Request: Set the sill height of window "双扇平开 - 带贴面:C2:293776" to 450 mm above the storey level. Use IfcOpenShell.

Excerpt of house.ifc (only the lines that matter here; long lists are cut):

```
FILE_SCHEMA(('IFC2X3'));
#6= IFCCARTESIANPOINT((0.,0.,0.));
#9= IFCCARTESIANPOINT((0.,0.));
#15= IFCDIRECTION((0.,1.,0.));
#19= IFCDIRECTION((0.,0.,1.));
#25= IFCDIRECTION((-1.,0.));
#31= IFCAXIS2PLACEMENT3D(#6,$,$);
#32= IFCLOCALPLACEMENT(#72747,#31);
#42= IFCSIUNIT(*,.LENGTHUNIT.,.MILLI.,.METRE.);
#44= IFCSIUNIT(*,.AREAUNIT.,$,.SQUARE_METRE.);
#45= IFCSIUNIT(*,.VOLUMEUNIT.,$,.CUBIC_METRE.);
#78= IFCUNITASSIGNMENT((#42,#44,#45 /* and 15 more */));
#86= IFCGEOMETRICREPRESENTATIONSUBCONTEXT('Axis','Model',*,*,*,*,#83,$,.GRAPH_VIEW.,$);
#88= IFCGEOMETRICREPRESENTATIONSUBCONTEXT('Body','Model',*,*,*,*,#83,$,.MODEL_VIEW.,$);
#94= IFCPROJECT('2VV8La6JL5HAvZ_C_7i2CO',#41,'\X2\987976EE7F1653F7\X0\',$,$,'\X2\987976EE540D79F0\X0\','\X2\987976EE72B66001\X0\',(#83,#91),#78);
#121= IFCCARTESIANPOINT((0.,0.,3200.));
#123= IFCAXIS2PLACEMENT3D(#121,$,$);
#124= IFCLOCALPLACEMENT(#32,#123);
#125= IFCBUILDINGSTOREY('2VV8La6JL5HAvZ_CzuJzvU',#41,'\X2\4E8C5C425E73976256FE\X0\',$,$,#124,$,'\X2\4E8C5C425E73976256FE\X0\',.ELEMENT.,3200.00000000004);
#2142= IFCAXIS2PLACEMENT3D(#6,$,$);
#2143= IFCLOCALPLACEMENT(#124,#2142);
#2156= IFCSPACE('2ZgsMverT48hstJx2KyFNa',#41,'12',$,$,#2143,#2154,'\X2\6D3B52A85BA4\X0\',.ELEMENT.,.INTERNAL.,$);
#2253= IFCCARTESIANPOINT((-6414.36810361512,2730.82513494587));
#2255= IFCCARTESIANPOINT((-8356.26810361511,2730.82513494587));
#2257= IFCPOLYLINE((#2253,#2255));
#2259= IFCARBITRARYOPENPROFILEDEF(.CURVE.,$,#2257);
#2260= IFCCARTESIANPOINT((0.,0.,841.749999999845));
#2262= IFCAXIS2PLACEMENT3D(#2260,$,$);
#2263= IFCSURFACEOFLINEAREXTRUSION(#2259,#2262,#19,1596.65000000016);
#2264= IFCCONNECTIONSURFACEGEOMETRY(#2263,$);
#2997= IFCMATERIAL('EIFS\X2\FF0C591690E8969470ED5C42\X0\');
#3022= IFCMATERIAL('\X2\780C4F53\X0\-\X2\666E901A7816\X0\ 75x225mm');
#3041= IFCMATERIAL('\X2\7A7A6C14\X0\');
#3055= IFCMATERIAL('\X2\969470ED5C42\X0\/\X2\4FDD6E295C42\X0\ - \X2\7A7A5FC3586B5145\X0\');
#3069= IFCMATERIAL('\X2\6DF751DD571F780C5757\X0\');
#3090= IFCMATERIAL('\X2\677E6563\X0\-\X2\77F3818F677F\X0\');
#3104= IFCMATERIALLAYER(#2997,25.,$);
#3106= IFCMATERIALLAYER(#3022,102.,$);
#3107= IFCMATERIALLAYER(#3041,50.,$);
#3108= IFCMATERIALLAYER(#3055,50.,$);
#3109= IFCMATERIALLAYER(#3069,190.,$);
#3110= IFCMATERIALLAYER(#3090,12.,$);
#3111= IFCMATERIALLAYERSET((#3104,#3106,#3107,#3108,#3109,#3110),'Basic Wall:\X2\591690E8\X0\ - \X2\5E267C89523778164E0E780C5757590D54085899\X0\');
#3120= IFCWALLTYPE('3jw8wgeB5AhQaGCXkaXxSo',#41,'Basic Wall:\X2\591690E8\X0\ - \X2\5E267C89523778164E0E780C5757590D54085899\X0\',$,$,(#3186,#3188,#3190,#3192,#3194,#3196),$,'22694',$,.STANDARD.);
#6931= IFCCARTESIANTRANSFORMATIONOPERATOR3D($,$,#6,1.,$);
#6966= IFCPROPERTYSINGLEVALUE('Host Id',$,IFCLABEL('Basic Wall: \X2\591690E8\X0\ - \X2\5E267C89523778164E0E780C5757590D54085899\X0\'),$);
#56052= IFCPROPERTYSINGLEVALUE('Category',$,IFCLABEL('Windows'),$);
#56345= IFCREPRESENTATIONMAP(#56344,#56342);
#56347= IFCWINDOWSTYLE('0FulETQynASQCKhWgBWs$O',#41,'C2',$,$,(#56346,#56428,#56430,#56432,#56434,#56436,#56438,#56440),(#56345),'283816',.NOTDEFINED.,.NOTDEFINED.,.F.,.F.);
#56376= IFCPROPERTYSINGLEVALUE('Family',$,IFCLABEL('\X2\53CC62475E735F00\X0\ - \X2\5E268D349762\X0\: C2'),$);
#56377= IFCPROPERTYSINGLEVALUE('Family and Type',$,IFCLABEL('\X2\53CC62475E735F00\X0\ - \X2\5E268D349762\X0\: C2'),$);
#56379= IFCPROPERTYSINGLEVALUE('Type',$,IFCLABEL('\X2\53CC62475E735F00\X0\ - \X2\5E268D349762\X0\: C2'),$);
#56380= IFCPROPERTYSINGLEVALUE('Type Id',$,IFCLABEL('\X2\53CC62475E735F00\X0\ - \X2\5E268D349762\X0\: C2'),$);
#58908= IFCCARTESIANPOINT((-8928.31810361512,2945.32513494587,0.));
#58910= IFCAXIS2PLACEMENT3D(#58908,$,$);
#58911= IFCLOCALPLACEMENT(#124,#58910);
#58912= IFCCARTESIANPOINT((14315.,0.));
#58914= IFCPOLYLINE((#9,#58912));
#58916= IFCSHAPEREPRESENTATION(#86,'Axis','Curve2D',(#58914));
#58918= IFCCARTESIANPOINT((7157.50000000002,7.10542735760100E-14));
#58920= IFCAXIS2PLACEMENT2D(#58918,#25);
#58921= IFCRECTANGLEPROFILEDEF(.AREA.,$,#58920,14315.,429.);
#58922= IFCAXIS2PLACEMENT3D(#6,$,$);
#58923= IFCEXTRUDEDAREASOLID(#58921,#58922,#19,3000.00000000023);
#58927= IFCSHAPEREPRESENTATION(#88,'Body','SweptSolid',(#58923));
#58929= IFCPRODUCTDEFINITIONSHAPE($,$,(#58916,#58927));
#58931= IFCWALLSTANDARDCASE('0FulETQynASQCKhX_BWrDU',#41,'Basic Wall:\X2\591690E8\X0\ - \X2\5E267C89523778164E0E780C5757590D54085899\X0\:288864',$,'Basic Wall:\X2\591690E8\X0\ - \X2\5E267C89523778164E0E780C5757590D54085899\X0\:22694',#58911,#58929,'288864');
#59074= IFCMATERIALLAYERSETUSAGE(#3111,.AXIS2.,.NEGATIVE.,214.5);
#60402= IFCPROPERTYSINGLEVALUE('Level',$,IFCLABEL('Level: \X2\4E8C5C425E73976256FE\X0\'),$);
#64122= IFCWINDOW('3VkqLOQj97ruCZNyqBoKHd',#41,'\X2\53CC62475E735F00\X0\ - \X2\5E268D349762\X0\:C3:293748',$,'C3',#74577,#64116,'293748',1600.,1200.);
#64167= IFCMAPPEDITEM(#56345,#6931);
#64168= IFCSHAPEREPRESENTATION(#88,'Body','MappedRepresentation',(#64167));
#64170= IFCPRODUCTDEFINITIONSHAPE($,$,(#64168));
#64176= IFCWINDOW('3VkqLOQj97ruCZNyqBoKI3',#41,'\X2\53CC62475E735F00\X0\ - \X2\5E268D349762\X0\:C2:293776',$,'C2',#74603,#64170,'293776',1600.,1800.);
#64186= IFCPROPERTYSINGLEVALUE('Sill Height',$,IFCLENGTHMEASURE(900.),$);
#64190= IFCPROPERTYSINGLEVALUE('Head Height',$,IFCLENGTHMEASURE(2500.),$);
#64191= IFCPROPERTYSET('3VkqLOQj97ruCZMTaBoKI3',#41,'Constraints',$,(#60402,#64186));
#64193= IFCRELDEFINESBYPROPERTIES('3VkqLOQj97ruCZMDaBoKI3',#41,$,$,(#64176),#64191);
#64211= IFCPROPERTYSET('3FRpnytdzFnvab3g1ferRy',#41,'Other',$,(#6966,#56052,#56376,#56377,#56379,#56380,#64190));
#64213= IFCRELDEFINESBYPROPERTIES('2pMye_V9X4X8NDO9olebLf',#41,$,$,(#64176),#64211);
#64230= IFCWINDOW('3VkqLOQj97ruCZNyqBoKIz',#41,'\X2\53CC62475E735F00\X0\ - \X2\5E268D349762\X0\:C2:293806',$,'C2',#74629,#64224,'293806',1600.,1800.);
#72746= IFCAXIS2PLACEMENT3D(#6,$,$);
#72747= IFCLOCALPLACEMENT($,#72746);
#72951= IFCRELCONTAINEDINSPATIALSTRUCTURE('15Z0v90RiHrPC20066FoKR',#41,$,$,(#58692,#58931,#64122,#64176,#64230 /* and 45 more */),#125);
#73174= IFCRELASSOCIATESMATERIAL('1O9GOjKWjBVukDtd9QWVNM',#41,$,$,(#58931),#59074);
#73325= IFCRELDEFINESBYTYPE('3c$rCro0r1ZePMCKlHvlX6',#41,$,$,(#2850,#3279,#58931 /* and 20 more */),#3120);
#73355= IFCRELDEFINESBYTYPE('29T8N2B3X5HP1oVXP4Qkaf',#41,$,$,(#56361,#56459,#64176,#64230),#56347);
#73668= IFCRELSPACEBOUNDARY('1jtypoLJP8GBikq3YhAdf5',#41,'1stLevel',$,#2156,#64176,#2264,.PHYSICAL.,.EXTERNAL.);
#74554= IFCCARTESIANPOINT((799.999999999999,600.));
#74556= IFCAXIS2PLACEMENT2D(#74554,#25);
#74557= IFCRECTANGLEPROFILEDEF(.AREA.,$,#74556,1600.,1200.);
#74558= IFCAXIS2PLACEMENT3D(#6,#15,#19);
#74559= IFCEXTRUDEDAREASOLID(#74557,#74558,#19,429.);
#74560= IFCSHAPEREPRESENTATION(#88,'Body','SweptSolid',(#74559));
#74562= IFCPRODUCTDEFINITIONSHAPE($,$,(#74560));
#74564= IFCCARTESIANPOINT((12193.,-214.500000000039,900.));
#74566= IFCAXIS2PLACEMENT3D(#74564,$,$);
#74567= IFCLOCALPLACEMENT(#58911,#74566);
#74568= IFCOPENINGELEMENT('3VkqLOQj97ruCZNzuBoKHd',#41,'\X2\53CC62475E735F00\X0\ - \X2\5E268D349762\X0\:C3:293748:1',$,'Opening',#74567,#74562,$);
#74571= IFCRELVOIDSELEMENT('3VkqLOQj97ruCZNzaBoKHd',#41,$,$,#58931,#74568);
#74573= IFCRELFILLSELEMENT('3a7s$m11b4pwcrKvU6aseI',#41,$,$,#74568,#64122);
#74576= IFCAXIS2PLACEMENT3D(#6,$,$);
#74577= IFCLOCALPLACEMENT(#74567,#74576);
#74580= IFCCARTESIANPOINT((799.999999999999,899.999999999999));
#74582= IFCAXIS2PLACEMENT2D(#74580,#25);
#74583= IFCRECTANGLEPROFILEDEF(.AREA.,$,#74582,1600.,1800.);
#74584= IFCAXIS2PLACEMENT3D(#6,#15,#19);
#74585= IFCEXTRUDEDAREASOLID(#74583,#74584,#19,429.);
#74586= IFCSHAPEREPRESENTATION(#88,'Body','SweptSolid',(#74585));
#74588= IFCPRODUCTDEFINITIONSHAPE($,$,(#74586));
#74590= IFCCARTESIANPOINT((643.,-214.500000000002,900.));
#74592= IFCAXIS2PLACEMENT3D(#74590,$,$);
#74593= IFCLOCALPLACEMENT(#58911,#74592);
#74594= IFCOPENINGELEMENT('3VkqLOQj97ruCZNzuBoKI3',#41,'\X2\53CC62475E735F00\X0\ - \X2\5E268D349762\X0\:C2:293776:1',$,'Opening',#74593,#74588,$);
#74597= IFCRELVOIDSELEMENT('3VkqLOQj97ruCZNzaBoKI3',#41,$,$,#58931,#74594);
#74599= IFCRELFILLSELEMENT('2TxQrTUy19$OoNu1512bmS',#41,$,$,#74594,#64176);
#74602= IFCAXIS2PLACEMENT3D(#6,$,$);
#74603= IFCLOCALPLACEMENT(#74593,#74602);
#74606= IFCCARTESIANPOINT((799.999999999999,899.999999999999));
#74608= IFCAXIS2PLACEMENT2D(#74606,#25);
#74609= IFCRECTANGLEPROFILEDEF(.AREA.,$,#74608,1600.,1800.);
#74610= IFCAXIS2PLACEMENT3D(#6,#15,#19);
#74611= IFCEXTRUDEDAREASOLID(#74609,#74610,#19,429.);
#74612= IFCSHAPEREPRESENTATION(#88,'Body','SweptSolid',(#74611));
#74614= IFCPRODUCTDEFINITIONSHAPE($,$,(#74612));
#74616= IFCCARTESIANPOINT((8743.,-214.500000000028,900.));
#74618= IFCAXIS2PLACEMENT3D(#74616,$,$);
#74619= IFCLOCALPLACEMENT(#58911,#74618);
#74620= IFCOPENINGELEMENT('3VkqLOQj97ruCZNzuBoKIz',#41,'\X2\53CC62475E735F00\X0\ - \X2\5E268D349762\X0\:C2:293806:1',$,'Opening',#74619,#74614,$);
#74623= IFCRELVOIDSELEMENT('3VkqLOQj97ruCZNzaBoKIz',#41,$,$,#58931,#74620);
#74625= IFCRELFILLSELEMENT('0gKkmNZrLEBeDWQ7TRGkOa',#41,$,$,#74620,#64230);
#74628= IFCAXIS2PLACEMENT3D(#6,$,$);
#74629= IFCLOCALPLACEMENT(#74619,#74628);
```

```python
import numpy as np
import ifcopenshell
import ifcopenshell.api.geometry
import ifcopenshell.api.pset
import ifcopenshell.geom
import ifcopenshell.util.element
import ifcopenshell.util.placement
import ifcopenshell.util.shape
import ifcopenshell.util.unit

model = ifcopenshell.open("house.ifc")
unit_scale = ifcopenshell.util.unit.calculate_unit_scale(model)

window = model.by_guid("3VkqLOQj97ruCZNyqBoKI3")
opening = window.FillsVoids[0].RelatingOpeningElement
storey = ifcopenshell.util.element.get_container(window, ifc_class="IfcBuildingStorey")
level = ifcopenshell.util.placement.get_local_placement(storey.ObjectPlacement)[2, 3]

# The opening's origin need not be at the sill, so measure its lowest point.
shape = ifcopenshell.geom.create_shape(ifcopenshell.geom.settings(), opening)
bottom = ifcopenshell.util.shape.get_shape_bottom_elevation(shape, shape.geometry) / unit_scale
dz = level + 0.45 / unit_scale - bottom

shift = np.array([0.0, 0.0, dz])
# The window is placed relative to its opening, so it follows when the opening moves.
matrix = ifcopenshell.util.placement.get_local_placement(opening.ObjectPlacement)
matrix[:3, 3] += shift
ifcopenshell.api.geometry.edit_object_placement(
    model, product=opening, matrix=matrix, is_si=False, should_transform_children=True
)

# Space boundary surfaces are stored in each space's coordinates; move them too.
for rel in window.ProvidesBoundaries:
    if not rel.ConnectionGeometry:
        continue
    surface = rel.ConnectionGeometry.SurfaceOnRelatingElement
    space_matrix = ifcopenshell.util.placement.get_local_placement(rel.RelatingSpace.ObjectPlacement)
    point = np.array(surface.Position.Location.Coordinates) + space_matrix[:3, :3].T @ shift
    surface.Position = model.createIfcAxis2Placement3D(
        model.createIfcCartesianPoint(point.tolist()), surface.Position.Axis, surface.Position.RefDirection
    )

# Keep the stored heights in step.
pset = model.by_id(ifcopenshell.util.element.get_pset(window, "Constraints", should_inherit=False)["id"])
ifcopenshell.api.pset.edit_pset(model, pset=pset, properties={
    "Sill Height": model.create_entity("IfcLengthMeasure", ifcopenshell.util.element.get_pset(window, "Constraints", "Sill Height") + dz),
})
pset = model.by_id(ifcopenshell.util.element.get_pset(window, "Other", should_inherit=False)["id"])
ifcopenshell.api.pset.edit_pset(model, pset=pset, properties={
    "Head Height": model.create_entity("IfcLengthMeasure", ifcopenshell.util.element.get_pset(window, "Other", "Head Height") + dz),
})

print(f"moved by {dz * unit_scale:+.3f} m")

model.write("house_updated.ifc")
```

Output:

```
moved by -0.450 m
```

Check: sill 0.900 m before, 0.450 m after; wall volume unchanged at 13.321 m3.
